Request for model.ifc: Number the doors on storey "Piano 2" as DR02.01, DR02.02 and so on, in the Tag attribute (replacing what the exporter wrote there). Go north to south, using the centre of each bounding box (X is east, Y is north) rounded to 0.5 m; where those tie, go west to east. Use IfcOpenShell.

First a look at what the model holds.

```python
import ifcopenshell
import ifcopenshell.util.element
import ifcopenshell.util.placement

model = ifcopenshell.open("model.ifc")
print(model.schema)
storey = next(s for s in model.by_type("IfcBuildingStorey") if s.Name == "Piano 2")
doors = [e for e in ifcopenshell.util.element.get_decomposition(storey) if e.is_a("IfcDoor")]
for e in sorted(doors, key=lambda e: e.id()):
    origin = ifcopenshell.util.placement.get_local_placement(e.ObjectPlacement)[:3, 3]
    print(e.id(), e.Tag, e.Name, origin.round(2) + 0.0, sep=" | ")
```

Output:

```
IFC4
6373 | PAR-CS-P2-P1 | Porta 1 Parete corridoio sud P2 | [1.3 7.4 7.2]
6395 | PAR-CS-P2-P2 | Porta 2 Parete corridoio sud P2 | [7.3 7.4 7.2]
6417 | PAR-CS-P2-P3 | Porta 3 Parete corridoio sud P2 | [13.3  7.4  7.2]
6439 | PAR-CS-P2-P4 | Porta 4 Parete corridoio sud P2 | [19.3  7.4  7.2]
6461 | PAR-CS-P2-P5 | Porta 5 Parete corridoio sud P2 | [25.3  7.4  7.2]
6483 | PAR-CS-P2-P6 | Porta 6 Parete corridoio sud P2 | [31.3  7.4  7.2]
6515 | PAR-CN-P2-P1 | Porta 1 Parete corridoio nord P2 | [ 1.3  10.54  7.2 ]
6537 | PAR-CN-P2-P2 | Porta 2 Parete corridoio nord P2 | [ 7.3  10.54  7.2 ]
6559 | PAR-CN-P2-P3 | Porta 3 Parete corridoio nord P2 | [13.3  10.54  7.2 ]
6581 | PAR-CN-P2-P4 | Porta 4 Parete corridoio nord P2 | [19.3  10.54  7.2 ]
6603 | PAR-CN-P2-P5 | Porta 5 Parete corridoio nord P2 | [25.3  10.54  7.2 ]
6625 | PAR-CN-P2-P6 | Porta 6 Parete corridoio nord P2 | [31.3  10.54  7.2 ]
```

```python
import ifcopenshell
import ifcopenshell.geom
import ifcopenshell.util.element
import ifcopenshell.util.shape

model = ifcopenshell.open("model.ifc")
settings = ifcopenshell.geom.settings()
settings.set("use-world-coords", True)


def centre(element):
    shape = ifcopenshell.geom.create_shape(settings, element)
    return ifcopenshell.util.shape.get_bbox_centroid(shape.geometry)


storey = next(s for s in model.by_type("IfcBuildingStorey") if s.Name == "Piano 2")
doors = [e for e in ifcopenshell.util.element.get_decomposition(storey) if e.is_a("IfcDoor")]

# Insertion points can sit at a corner or the storey origin, so sort by the geometry (in metres).
centres = {e: centre(e) for e in doors}
doors.sort(key=lambda e: (-round(centres[e][1] / 0.5), centres[e][0]))

for i, e in enumerate(doors, start=1):
    number = f"DR02.{i:02d}"
    e.Tag = number
    print(e.id(), number)

model.write("model_rev.ifc")
```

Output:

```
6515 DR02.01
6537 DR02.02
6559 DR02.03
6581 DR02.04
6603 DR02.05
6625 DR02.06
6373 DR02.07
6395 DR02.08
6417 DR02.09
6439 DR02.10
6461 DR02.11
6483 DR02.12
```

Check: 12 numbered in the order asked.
